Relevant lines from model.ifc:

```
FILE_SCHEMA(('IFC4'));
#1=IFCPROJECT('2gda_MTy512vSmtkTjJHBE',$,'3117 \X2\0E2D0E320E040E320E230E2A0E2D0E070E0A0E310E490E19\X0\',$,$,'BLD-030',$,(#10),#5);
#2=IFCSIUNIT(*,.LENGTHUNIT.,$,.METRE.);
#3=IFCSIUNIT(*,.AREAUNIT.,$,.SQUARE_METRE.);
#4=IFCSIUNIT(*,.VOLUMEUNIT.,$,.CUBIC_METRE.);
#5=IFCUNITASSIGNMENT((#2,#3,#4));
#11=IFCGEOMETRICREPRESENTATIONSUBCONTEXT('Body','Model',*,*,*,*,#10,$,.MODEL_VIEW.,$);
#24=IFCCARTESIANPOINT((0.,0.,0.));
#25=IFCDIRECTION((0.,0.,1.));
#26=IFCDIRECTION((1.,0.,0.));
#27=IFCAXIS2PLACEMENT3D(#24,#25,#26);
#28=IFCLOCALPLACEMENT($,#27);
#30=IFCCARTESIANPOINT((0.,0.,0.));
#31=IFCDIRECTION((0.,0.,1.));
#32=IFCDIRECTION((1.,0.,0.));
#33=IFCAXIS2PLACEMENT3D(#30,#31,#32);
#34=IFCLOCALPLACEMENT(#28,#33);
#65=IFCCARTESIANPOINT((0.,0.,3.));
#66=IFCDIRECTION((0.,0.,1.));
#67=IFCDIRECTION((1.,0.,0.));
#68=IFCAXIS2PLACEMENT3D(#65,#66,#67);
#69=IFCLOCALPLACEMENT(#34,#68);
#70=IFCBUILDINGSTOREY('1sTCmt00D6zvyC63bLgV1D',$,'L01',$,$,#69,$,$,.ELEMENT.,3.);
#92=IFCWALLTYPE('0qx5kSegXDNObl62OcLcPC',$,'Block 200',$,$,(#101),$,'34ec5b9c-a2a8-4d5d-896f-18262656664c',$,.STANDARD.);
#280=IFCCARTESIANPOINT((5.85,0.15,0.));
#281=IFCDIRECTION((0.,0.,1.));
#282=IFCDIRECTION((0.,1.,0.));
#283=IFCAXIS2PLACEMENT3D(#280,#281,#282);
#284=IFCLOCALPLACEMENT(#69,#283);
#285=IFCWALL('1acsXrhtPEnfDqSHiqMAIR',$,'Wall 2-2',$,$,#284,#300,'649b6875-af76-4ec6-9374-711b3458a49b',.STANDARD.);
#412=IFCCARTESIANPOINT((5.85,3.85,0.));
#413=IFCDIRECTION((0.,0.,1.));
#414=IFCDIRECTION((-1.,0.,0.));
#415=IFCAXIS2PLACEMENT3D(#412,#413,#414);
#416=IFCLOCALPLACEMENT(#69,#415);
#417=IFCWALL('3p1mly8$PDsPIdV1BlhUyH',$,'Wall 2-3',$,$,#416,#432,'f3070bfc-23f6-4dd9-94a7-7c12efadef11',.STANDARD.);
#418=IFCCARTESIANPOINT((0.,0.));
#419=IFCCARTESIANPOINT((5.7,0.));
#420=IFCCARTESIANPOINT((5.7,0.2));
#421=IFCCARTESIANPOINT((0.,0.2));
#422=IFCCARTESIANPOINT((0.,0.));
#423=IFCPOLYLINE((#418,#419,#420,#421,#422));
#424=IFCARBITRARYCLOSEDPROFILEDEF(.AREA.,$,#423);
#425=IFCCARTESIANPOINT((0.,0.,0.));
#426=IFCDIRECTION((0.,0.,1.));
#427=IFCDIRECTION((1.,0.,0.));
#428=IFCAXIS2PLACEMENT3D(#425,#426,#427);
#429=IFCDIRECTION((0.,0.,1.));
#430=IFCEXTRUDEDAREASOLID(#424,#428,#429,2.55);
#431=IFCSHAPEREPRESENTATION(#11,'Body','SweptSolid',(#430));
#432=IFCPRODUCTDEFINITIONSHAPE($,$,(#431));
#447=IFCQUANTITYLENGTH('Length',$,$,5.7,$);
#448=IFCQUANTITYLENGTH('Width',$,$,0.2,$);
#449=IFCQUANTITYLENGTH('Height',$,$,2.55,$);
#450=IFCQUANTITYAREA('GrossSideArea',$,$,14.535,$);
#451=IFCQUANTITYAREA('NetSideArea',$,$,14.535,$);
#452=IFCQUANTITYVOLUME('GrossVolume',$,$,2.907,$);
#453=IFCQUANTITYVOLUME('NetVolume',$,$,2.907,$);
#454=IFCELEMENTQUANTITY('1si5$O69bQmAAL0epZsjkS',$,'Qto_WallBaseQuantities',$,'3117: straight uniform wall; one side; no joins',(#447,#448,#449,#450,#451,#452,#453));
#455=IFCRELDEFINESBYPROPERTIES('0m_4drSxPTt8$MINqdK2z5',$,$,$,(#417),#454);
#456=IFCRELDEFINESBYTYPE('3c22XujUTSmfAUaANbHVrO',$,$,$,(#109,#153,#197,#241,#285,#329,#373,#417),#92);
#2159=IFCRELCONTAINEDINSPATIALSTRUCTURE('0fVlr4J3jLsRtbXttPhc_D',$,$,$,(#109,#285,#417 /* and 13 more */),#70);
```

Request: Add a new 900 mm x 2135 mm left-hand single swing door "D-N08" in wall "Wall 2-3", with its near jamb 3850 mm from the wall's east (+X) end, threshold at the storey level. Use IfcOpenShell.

```python
import numpy as np
import ifcopenshell
import ifcopenshell.api.feature
import ifcopenshell.api.geometry
import ifcopenshell.api.pset
import ifcopenshell.api.root
import ifcopenshell.api.spatial
import ifcopenshell.geom
import ifcopenshell.util.element
import ifcopenshell.util.placement
import ifcopenshell.util.representation
import ifcopenshell.util.shape
import ifcopenshell.util.unit

model = ifcopenshell.open("model.ifc")
unit_scale = ifcopenshell.util.unit.calculate_unit_scale(model)
area_scale = ifcopenshell.util.unit.calculate_unit_scale(model, "AREAUNIT")
volume_scale = ifcopenshell.util.unit.calculate_unit_scale(model, "VOLUMEUNIT")
settings = ifcopenshell.geom.settings()


def volume(element):
    """Net volume in cubic metres, openings subtracted."""
    shape = ifcopenshell.geom.create_shape(settings, element)
    return ifcopenshell.util.shape.get_volume(shape.geometry)


wall = model.by_id(417)
storey = ifcopenshell.util.element.get_container(wall, ifc_class="IfcBuildingStorey")
context = ifcopenshell.util.representation.get_context(model, "Model", "Body", "MODEL_VIEW")
before = volume(wall)

width, height, from_end, sill = 0.9, 2.135, 3.85, 0.0  # metres

# The wall runs along its own X axis, and the end named is its -X end.
wall_shape = ifcopenshell.geom.create_shape(settings, wall)
x, y, z = ifcopenshell.util.shape.get_vertices(wall_shape.geometry).T
start = x.min() + from_end
face, thickness = float(y.min()), float(y.max() - y.min())
wall_matrix = ifcopenshell.util.placement.get_local_placement(wall.ObjectPlacement)
level = ifcopenshell.util.placement.get_local_placement(storey.ObjectPlacement)[2, 3]


def in_wall(x, y):
    """Placement at x, y metres in the wall's axes, at sill height."""
    matrix = wall_matrix.copy()
    matrix[:, 3] = wall_matrix @ np.array([x / unit_scale, y / unit_scale, 0.0, 1.0])
    matrix[2, 3] = level + sill / unit_scale
    return matrix


# Opening: a box that overshoots both wall faces by 50 mm.
opening = ifcopenshell.api.root.create_entity(model, ifc_class="IfcOpeningElement", predefined_type="OPENING")
box = ifcopenshell.api.geometry.add_wall_representation(
    model, context=context, length=width, height=height, thickness=thickness + 0.1
)
ifcopenshell.api.geometry.assign_representation(model, product=opening, representation=box)
ifcopenshell.api.geometry.edit_object_placement(model, product=opening, matrix=in_wall(start, face - 0.05), is_si=False)
ifcopenshell.api.feature.add_feature(model, feature=opening, element=wall)

door = ifcopenshell.api.root.create_entity(model, ifc_class="IfcDoor", name="D-N08", predefined_type="DOOR")
door.OverallWidth, door.OverallHeight = width / unit_scale, height / unit_scale
door.OperationType = "SINGLE_SWING_LEFT"
body = ifcopenshell.api.geometry.add_door_representation(
    model,
    context=context,
    overall_width=door.OverallWidth,
    overall_height=door.OverallHeight,
    operation_type="SINGLE_SWING_LEFT",
    lining_properties={"LiningDepth": thickness / unit_scale, "ThresholdDepth": thickness / unit_scale},
)
ifcopenshell.api.geometry.assign_representation(model, product=door, representation=body)
ifcopenshell.api.spatial.assign_container(model, products=[door], relating_structure=storey)
ifcopenshell.api.feature.add_filling(model, opening=opening, element=door)

# The lining spans the wall, so the door starts at the wall face.
ifcopenshell.api.geometry.edit_object_placement(model, product=door, matrix=in_wall(start, face), is_si=False)

after = volume(wall)

# Update the wall's stored quantities.
qto = model.by_id(ifcopenshell.util.element.get_pset(wall, "Qto_WallBaseQuantities", should_inherit=False)["id"])
ifcopenshell.api.pset.edit_qto(model, qto=qto, properties={
    "NetSideArea": after / thickness / area_scale,
    "NetVolume": after / volume_scale,
})

print(f"wall volume {before:.3f} -> {after:.3f} m3")

model.write("model_rev.ifc")
```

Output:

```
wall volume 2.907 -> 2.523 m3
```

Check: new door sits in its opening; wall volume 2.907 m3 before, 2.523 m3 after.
